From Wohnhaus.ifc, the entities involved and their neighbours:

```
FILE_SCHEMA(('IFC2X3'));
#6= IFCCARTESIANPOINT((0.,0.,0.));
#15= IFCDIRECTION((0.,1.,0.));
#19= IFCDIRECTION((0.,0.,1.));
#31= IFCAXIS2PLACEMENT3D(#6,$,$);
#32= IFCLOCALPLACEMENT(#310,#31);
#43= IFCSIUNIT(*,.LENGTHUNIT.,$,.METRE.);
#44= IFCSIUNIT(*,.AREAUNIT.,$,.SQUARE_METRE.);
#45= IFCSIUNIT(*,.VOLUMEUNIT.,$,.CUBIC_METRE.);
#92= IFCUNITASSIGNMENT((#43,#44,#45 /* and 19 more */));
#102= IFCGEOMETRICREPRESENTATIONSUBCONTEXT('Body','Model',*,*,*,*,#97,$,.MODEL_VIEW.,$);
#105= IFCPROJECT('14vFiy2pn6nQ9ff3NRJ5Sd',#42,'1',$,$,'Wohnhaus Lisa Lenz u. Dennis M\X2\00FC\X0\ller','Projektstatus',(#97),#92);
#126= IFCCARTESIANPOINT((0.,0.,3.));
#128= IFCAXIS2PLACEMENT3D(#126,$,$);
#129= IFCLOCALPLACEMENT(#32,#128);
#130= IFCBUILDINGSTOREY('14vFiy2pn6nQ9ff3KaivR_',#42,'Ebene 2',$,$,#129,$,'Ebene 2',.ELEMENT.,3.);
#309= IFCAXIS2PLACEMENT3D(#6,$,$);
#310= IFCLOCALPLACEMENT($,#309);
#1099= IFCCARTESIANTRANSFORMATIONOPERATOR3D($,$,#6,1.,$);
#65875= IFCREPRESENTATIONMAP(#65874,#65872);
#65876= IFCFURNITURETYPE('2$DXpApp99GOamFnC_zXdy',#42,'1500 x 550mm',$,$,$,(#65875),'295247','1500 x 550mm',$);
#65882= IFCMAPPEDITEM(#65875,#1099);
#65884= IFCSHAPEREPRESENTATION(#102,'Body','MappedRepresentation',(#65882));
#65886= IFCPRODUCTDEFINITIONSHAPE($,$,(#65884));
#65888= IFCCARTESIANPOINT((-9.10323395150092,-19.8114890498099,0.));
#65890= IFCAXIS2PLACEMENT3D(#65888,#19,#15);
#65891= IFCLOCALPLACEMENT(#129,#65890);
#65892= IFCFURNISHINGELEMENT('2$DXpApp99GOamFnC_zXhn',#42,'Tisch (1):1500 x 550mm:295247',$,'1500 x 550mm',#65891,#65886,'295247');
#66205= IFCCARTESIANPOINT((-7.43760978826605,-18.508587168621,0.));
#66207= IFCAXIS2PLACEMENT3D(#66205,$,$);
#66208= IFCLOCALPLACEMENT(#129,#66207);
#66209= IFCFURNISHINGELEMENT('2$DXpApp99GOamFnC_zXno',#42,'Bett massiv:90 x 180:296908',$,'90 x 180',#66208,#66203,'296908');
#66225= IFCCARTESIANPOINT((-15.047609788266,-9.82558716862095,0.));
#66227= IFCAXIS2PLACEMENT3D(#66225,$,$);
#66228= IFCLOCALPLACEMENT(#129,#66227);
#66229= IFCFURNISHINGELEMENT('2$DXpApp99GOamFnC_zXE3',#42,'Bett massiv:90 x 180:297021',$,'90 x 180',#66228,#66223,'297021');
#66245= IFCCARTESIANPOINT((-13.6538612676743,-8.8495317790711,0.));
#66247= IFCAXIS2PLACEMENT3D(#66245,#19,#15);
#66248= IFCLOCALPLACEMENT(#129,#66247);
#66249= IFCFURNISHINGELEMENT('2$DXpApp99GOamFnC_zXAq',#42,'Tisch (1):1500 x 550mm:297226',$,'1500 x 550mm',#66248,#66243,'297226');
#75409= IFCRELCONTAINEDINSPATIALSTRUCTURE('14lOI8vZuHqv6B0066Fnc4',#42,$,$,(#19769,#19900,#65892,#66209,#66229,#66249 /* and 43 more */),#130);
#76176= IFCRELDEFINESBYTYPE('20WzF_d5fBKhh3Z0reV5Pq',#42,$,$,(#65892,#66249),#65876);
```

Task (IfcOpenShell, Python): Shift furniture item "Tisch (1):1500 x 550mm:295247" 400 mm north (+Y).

```python
import ifcopenshell
import ifcopenshell.api.geometry
import ifcopenshell.util.placement
import ifcopenshell.util.unit

model = ifcopenshell.open("Wohnhaus.ifc")
unit_scale = ifcopenshell.util.unit.calculate_unit_scale(model)

item = model.by_id(65892)
matrix = ifcopenshell.util.placement.get_local_placement(item.ObjectPlacement)
matrix[1, 3] += 0.4 / unit_scale
ifcopenshell.api.geometry.edit_object_placement(model, product=item, matrix=matrix, is_si=False)

print(ifcopenshell.util.placement.get_local_placement(item.ObjectPlacement).round(3) + 0.0)

model.write("Wohnhaus_v2.ifc")
```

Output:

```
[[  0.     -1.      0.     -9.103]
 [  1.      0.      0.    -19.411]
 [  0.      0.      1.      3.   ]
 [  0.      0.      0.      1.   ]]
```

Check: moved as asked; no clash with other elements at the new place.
